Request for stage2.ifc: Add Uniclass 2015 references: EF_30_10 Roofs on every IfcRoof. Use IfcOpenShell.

First a look at what the model holds.

```python
import ifcopenshell

model = ifcopenshell.open("stage2.ifc")
print(model.schema)
print("classifications:", [c.Name for c in model.by_type("IfcClassification")])
for ifc_class in ("IfcDoor", "IfcRoof", "IfcStair", "IfcWall", "IfcWindow"):
    print(ifc_class, len(model.by_type(ifc_class)))
```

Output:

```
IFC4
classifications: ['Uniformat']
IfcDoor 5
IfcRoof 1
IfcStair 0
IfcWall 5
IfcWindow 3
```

```python
import ifcopenshell
import ifcopenshell.api.classification

model = ifcopenshell.open("stage2.ifc")

system = ifcopenshell.api.classification.add_classification(model, classification="Uniclass 2015")

codes = {
    "IfcRoof": ("EF_30_10", "Roofs"),
}
for ifc_class, (code, name) in codes.items():
    products = model.by_type(ifc_class)
    ifcopenshell.api.classification.add_reference(
        model, products=products, classification=system, identification=code, name=name
    )
    print(code, len(products))

model.write("stage2_edited.ifc")
```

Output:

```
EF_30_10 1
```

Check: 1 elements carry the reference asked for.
